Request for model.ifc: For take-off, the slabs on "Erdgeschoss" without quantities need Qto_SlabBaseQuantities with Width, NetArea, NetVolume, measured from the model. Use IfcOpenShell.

First a look at what the model holds.

```python
import ifcopenshell
import ifcopenshell.util.element
import ifcopenshell.util.unit

model = ifcopenshell.open("model.ifc")
print(model.schema)
for unit_type in ("LENGTHUNIT", "AREAUNIT", "VOLUMEUNIT"):
    print(unit_type, ifcopenshell.util.unit.calculate_unit_scale(model, unit_type))
storey = next(s for s in model.by_type("IfcBuildingStorey") if s.Name == "Erdgeschoss")
slabs = [e for e in ifcopenshell.util.element.get_decomposition(storey) if e.is_a("IfcSlab")]
for e in sorted(slabs, key=lambda e: e.id()):
    print(e.id(), e.is_a(), e.Name, list(ifcopenshell.util.element.get_psets(e, qtos_only=True)), sep=" | ")
```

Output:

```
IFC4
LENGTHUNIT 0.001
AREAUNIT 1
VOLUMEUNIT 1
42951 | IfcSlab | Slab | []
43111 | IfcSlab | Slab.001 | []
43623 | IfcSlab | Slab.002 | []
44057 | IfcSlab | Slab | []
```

```python
import ifcopenshell
import ifcopenshell.api.pset
import ifcopenshell.geom
import ifcopenshell.util.element
import ifcopenshell.util.shape
import ifcopenshell.util.unit

model = ifcopenshell.open("model.ifc")
unit_scale = ifcopenshell.util.unit.calculate_unit_scale(model)
area_scale = ifcopenshell.util.unit.calculate_unit_scale(model, "AREAUNIT")
volume_scale = ifcopenshell.util.unit.calculate_unit_scale(model, "VOLUMEUNIT")
settings = ifcopenshell.geom.settings()

storey = next(s for s in model.by_type("IfcBuildingStorey") if s.Name == "Erdgeschoss")
slabs = [e for e in ifcopenshell.util.element.get_decomposition(storey) if e.is_a("IfcSlab")]

for e in sorted(slabs, key=lambda e: e.id()):
    if ifcopenshell.util.element.get_psets(e, qtos_only=True, should_inherit=False):
        continue
    # Geometry comes back in metres, in the element's own axes.
    shape = ifcopenshell.geom.create_shape(settings, e)
    values = {
        "Width": ifcopenshell.util.shape.get_z(shape.geometry) / unit_scale,
        "NetArea": ifcopenshell.util.shape.get_footprint_area(shape.geometry) / area_scale,
        "NetVolume": ifcopenshell.util.shape.get_volume(shape.geometry) / volume_scale,
    }
    qto = ifcopenshell.api.pset.add_qto(model, product=e, name="Qto_SlabBaseQuantities")
    ifcopenshell.api.pset.edit_qto(model, qto=qto, properties=values)
    print(e.id(), {k: round(v, 3) for k, v in values.items()})

model.write("model-out.ifc")
```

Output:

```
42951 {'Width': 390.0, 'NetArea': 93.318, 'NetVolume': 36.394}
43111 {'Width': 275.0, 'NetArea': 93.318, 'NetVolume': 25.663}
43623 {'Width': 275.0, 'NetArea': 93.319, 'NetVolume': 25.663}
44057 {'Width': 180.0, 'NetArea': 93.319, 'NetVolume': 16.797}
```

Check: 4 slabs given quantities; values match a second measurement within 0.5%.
